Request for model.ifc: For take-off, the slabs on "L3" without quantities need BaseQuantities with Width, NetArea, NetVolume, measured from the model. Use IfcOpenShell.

First a look at what the model holds.

```python
import ifcopenshell
import ifcopenshell.util.element
import ifcopenshell.util.unit

model = ifcopenshell.open("model.ifc")
print(model.schema)
for unit_type in ("LENGTHUNIT", "AREAUNIT", "VOLUMEUNIT"):
    print(unit_type, ifcopenshell.util.unit.calculate_unit_scale(model, unit_type))
storey = next(s for s in model.by_type("IfcBuildingStorey") if s.Name == "L3")
slabs = [e for e in ifcopenshell.util.element.get_decomposition(storey) if e.is_a("IfcSlab")]
for e in sorted(slabs, key=lambda e: e.id()):
    print(e.id(), e.is_a(), e.Name, list(ifcopenshell.util.element.get_psets(e, qtos_only=True)), sep=" | ")
```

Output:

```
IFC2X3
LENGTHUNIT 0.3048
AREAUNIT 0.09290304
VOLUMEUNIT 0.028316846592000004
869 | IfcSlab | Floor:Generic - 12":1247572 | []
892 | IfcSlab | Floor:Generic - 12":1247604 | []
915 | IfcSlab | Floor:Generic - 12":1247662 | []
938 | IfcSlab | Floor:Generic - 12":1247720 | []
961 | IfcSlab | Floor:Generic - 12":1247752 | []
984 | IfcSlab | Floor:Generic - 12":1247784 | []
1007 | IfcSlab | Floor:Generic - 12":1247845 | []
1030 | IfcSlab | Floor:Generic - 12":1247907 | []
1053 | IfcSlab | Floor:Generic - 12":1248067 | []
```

```python
import ifcopenshell
import ifcopenshell.api.pset
import ifcopenshell.geom
import ifcopenshell.util.element
import ifcopenshell.util.shape
import ifcopenshell.util.unit

model = ifcopenshell.open("model.ifc")
unit_scale = ifcopenshell.util.unit.calculate_unit_scale(model)
area_scale = ifcopenshell.util.unit.calculate_unit_scale(model, "AREAUNIT")
volume_scale = ifcopenshell.util.unit.calculate_unit_scale(model, "VOLUMEUNIT")
settings = ifcopenshell.geom.settings()

storey = next(s for s in model.by_type("IfcBuildingStorey") if s.Name == "L3")
slabs = [e for e in ifcopenshell.util.element.get_decomposition(storey) if e.is_a("IfcSlab")]

for e in sorted(slabs, key=lambda e: e.id()):
    if ifcopenshell.util.element.get_psets(e, qtos_only=True, should_inherit=False):
        continue
    # Geometry comes back in metres, in the element's own axes.
    shape = ifcopenshell.geom.create_shape(settings, e)
    values = {
        "Width": ifcopenshell.util.shape.get_z(shape.geometry) / unit_scale,
        "NetArea": ifcopenshell.util.shape.get_footprint_area(shape.geometry) / area_scale,
        "NetVolume": ifcopenshell.util.shape.get_volume(shape.geometry) / volume_scale,
    }
    qto = ifcopenshell.api.pset.add_qto(model, product=e, name="BaseQuantities")
    ifcopenshell.api.pset.edit_qto(model, qto=qto, properties=values)
    print(e.id(), {k: round(v, 3) for k, v in values.items()})

model.write("model_updated.ifc")
```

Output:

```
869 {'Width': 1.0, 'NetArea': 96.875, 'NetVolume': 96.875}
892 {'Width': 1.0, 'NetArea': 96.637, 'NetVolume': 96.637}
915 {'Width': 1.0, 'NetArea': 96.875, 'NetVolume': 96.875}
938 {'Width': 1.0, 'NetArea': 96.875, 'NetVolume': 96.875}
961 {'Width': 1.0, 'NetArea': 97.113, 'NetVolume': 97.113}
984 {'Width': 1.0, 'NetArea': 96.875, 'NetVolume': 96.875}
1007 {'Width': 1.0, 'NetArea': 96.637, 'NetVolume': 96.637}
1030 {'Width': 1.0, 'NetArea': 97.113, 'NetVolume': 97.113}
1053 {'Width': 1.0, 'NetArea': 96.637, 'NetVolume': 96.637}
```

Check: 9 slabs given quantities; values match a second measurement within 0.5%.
